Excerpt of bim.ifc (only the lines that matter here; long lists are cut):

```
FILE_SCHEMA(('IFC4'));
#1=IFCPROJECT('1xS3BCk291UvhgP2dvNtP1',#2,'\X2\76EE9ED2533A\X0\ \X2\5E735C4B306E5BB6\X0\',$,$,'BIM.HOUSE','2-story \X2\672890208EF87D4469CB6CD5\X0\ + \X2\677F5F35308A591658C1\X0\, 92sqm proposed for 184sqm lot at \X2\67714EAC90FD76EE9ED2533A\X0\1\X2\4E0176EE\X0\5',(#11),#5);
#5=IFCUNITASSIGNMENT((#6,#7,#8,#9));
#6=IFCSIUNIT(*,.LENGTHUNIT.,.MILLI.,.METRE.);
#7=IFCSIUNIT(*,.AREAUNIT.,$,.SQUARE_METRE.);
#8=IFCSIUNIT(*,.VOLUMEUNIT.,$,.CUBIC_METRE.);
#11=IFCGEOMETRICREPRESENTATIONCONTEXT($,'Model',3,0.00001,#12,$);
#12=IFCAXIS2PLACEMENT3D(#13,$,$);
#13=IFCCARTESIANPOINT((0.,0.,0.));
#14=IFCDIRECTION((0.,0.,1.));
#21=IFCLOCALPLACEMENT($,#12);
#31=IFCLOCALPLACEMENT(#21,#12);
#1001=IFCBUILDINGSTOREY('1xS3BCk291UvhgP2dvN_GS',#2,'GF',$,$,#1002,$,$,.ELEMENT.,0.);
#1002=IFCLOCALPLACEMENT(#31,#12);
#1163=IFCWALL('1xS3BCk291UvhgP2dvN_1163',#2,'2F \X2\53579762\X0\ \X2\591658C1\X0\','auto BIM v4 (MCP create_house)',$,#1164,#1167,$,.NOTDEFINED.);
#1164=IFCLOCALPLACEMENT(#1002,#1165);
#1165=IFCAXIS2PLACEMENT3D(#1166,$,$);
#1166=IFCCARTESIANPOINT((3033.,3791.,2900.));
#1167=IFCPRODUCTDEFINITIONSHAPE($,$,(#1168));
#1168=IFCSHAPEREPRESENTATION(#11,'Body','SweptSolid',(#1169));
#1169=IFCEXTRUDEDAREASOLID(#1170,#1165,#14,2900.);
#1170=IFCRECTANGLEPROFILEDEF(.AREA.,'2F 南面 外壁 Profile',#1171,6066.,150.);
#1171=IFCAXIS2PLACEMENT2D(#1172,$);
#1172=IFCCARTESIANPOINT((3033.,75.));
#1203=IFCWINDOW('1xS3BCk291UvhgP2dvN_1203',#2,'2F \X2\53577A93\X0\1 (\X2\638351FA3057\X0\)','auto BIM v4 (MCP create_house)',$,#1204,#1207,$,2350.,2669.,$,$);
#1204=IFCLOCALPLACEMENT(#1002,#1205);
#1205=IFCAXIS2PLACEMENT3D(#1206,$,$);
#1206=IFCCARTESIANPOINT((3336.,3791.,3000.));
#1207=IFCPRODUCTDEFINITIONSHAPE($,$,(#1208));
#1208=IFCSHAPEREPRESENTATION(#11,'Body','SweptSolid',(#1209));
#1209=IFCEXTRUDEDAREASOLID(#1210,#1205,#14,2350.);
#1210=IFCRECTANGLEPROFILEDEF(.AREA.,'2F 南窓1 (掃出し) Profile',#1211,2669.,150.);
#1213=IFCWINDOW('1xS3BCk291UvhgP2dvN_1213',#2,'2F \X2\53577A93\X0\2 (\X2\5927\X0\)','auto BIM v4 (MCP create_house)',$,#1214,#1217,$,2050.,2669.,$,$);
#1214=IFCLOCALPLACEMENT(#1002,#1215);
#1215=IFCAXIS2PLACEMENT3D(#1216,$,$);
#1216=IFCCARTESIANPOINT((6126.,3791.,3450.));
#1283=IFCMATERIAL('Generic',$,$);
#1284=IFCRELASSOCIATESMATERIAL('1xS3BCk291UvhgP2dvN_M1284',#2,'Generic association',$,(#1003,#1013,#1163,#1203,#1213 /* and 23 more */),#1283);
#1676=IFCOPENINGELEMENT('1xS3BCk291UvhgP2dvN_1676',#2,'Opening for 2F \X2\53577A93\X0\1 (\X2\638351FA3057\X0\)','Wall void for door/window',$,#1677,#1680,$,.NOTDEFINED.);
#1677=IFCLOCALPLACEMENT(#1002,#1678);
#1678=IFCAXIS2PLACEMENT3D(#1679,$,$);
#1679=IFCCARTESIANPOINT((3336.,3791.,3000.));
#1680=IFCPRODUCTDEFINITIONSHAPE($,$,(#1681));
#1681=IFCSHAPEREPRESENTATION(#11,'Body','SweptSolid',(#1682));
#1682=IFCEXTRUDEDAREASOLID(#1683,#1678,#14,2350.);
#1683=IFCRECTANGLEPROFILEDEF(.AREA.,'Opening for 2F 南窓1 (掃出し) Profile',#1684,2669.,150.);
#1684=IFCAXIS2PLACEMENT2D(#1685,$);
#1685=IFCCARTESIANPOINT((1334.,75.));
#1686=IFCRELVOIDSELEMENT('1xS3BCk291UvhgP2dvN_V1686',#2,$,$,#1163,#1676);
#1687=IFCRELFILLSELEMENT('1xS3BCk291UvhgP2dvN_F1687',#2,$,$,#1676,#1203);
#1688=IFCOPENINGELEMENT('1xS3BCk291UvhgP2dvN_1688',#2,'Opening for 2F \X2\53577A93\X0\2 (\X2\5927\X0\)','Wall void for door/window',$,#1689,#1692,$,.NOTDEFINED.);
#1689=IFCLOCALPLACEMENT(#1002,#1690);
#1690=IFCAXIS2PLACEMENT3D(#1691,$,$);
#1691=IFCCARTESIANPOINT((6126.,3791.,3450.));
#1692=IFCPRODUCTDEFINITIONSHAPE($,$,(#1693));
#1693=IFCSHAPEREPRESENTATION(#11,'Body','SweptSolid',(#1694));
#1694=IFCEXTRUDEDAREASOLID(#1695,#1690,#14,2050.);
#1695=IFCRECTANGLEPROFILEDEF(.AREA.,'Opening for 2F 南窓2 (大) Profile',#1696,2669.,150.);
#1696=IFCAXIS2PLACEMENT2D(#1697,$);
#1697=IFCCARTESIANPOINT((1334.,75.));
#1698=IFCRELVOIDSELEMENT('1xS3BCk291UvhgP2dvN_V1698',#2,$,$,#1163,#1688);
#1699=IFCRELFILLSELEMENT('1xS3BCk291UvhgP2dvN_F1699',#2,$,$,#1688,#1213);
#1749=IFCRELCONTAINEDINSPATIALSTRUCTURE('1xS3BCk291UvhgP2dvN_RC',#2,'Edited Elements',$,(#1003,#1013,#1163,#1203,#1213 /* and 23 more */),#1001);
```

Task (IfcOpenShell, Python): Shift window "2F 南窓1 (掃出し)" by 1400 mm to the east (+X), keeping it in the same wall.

```python
import ifcopenshell
import ifcopenshell.api.geometry
import ifcopenshell.util.placement
import ifcopenshell.util.unit

model = ifcopenshell.open("bim.ifc")
unit_scale = ifcopenshell.util.unit.calculate_unit_scale(model)

window = model.by_guid("1xS3BCk291UvhgP2dvN_1203")
opening = window.FillsVoids[0].RelatingOpeningElement
wall = opening.VoidsElements[0].RelatingBuildingElement

wall_matrix = ifcopenshell.util.placement.get_local_placement(wall.ObjectPlacement)
shift = wall_matrix[:3, 0] * 1.4 / unit_scale
before = ifcopenshell.util.placement.get_local_placement(window.ObjectPlacement)[:3, 3].copy()

# The window is not placed relative to its opening, so move both.
for product in (opening, window):
    matrix = ifcopenshell.util.placement.get_local_placement(product.ObjectPlacement)
    matrix[:3, 3] += shift
    ifcopenshell.api.geometry.edit_object_placement(model, product=product, matrix=matrix, is_si=False)

after = ifcopenshell.util.placement.get_local_placement(window.ObjectPlacement)[:3, 3]
print("window moved by", (after - before).round(3) + 0.0)

model.write("bim_updated.ifc")
```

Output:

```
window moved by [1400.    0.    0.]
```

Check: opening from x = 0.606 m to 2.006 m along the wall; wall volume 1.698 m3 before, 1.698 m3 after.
